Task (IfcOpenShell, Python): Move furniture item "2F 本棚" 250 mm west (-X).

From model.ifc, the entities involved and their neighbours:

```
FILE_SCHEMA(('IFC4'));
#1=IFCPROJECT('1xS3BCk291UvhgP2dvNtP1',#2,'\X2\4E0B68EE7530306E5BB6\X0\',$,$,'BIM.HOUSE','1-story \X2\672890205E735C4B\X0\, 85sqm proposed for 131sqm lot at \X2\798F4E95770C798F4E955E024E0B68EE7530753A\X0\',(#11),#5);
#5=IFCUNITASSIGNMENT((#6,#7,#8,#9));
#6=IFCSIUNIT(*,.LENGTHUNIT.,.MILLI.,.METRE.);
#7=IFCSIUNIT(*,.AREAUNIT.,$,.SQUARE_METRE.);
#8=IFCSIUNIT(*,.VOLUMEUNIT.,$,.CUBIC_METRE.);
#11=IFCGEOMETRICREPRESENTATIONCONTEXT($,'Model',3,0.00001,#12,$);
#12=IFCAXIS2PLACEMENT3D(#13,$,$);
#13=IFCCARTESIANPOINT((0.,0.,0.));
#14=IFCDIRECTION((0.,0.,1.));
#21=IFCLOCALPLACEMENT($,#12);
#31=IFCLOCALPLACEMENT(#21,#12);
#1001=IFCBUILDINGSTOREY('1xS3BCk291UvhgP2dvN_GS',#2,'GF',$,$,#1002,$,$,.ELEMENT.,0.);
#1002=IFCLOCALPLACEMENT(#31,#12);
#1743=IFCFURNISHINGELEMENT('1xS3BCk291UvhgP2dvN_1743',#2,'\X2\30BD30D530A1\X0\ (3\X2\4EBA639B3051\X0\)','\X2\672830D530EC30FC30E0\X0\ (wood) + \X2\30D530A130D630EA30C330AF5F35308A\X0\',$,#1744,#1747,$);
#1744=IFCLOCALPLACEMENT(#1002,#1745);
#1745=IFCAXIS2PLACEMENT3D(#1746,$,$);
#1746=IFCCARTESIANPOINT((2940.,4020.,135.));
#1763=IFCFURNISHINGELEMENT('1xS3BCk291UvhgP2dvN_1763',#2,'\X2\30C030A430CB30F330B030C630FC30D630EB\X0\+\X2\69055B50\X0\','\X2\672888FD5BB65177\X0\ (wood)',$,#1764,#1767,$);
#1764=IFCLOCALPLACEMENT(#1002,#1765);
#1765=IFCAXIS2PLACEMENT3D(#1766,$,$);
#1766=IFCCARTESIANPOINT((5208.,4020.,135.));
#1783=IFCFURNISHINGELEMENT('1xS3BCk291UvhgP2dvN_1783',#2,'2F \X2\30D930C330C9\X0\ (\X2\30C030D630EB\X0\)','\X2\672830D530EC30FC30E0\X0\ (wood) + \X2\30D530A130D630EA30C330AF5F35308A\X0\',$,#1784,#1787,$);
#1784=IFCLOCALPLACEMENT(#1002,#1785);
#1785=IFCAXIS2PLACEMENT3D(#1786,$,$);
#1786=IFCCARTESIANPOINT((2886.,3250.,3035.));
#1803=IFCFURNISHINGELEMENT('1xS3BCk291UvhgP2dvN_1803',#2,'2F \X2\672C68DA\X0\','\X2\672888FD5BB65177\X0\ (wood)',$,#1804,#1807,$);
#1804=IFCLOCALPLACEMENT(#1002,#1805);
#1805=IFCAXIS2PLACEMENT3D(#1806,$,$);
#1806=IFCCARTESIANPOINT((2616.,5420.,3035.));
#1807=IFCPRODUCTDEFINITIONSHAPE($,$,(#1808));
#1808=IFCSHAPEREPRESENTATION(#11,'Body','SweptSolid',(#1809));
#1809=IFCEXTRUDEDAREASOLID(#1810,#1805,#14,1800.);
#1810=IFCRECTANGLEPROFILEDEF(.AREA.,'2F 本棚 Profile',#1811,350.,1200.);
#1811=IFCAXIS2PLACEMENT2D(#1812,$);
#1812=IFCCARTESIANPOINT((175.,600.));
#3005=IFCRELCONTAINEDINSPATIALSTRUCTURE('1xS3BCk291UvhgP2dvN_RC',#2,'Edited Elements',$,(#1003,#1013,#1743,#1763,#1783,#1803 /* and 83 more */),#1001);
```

```python
import ifcopenshell
import ifcopenshell.api.geometry
import ifcopenshell.util.placement

model = ifcopenshell.open("model.ifc")

item = model.by_guid("1xS3BCk291UvhgP2dvN_1803")
matrix = ifcopenshell.util.placement.get_local_placement(item.ObjectPlacement)
matrix[0, 3] -= 250.0
ifcopenshell.api.geometry.edit_object_placement(model, product=item, matrix=matrix, is_si=False)

print(ifcopenshell.util.placement.get_local_placement(item.ObjectPlacement).round(3) + 0.0)

model.write("model_rev.ifc")
```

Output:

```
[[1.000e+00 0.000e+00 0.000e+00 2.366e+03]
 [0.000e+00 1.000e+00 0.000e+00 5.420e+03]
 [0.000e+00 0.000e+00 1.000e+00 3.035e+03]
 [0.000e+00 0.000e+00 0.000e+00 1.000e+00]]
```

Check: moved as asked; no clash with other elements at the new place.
